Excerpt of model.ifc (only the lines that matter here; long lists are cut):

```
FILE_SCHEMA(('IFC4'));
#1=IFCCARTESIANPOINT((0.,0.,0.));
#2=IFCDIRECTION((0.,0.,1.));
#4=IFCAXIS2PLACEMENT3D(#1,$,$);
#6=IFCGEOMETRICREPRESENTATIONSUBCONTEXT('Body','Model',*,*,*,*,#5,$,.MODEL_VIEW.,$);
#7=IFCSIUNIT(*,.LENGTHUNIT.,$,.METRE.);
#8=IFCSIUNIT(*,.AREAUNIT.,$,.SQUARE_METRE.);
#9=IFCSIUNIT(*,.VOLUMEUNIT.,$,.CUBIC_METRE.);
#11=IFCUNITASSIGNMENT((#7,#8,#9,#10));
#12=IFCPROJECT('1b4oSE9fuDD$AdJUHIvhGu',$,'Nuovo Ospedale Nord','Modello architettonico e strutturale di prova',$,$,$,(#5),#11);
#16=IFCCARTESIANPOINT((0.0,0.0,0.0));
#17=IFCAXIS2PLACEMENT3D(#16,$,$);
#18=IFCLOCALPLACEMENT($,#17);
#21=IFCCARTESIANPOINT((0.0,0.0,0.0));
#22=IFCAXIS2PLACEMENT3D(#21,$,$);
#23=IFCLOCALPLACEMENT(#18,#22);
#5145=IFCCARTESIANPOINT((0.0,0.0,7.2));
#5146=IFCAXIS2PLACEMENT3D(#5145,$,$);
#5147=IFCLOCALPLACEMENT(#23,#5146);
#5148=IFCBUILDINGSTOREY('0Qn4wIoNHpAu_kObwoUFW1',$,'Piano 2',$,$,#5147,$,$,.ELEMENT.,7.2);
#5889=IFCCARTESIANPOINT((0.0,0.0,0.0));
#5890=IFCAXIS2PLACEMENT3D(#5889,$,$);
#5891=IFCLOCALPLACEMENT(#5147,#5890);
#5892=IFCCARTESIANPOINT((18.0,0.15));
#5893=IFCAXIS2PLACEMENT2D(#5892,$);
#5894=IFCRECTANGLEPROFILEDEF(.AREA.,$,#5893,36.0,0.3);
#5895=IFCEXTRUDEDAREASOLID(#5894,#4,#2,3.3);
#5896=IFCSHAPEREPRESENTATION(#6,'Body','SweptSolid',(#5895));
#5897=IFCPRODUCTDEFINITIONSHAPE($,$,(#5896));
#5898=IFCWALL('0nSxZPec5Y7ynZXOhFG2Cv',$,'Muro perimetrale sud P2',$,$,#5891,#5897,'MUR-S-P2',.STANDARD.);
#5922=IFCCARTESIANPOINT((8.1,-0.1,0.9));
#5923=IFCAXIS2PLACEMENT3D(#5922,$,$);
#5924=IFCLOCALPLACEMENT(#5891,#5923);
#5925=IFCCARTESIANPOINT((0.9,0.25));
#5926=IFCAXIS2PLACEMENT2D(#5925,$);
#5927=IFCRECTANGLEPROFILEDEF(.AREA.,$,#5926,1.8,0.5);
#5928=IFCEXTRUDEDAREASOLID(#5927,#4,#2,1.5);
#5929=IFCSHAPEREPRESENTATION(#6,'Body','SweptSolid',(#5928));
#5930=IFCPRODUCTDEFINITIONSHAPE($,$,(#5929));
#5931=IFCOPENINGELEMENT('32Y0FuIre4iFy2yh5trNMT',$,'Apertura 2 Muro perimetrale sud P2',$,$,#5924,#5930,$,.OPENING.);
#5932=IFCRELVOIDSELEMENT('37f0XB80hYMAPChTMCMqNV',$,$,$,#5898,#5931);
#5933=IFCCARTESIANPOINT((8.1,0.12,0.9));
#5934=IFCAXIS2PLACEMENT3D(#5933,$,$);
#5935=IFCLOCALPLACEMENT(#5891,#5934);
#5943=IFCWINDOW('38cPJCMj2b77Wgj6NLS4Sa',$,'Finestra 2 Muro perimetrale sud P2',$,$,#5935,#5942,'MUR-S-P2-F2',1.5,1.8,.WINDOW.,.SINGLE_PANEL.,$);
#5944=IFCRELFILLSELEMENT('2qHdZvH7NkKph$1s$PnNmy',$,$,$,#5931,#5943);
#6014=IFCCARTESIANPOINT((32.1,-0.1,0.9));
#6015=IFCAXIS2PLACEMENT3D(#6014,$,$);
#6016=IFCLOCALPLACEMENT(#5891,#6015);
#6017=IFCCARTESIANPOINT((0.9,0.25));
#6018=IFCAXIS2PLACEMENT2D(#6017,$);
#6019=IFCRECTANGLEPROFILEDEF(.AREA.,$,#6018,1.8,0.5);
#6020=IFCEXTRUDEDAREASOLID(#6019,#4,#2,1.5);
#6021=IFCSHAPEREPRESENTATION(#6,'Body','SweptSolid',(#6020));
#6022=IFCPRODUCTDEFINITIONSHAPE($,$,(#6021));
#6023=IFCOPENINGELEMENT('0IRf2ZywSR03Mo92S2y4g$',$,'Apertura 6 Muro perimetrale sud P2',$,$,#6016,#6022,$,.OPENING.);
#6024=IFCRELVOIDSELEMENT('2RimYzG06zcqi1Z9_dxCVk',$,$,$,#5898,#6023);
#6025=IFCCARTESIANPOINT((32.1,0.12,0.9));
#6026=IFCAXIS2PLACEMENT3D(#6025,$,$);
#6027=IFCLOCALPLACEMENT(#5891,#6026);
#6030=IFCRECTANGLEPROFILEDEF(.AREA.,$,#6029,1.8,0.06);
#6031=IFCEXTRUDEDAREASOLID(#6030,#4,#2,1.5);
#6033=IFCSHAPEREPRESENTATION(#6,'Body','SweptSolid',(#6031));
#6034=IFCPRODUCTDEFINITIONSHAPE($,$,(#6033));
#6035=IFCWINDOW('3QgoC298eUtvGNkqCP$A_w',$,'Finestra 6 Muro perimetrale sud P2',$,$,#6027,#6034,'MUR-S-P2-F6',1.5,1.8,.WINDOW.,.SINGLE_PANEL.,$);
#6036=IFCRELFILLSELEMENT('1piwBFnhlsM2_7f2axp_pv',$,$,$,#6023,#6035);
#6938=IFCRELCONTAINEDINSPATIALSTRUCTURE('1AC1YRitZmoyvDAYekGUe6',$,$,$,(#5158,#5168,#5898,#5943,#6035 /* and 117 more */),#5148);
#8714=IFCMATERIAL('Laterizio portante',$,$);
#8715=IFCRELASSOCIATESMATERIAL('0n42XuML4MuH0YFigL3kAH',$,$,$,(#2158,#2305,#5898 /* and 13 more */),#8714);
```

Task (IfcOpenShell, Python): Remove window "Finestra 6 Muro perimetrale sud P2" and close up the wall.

```python
import ifcopenshell
import ifcopenshell.api.feature
import ifcopenshell.api.root
import ifcopenshell.geom
import ifcopenshell.util.shape

model = ifcopenshell.open("model.ifc")
settings = ifcopenshell.geom.settings()


def volume(element):
    """Net volume in cubic metres, openings subtracted."""
    shape = ifcopenshell.geom.create_shape(settings, element)
    return ifcopenshell.util.shape.get_volume(shape.geometry)


window = model.by_guid("3QgoC298eUtvGNkqCP$A_w")
opening = window.FillsVoids[0].RelatingOpeningElement
wall = opening.VoidsElements[0].RelatingBuildingElement
before = volume(wall)

ifcopenshell.api.root.remove_product(model, product=window)
ifcopenshell.api.feature.remove_feature(model, feature=opening)

after = volume(wall)

print(f"wall volume {before:.3f} -> {after:.3f} m3")

model.write("model_updated.ifc")
```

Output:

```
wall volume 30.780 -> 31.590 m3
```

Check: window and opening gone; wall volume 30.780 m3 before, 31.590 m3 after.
